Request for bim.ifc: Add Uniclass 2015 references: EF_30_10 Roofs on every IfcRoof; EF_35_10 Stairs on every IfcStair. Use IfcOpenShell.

First a look at what the model holds.

```python
import ifcopenshell

model = ifcopenshell.open("bim.ifc")
print(model.schema)
print("classifications:", [c.Name for c in model.by_type("IfcClassification")])
for ifc_class in ("IfcDoor", "IfcRoof", "IfcStair", "IfcWall", "IfcWindow"):
    print(ifc_class, len(model.by_type(ifc_class)))
```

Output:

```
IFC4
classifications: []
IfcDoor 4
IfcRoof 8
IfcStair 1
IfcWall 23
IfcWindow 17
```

```python
import ifcopenshell
import ifcopenshell.api.classification

model = ifcopenshell.open("bim.ifc")

system = ifcopenshell.api.classification.add_classification(model, classification="Uniclass 2015")

codes = {
    "IfcRoof": ("EF_30_10", "Roofs"),
    "IfcStair": ("EF_35_10", "Stairs"),
}
for ifc_class, (code, name) in codes.items():
    products = model.by_type(ifc_class)
    ifcopenshell.api.classification.add_reference(
        model, products=products, classification=system, identification=code, name=name
    )
    print(code, len(products))

model.write("bim_updated.ifc")
```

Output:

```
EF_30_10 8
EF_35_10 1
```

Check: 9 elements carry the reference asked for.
